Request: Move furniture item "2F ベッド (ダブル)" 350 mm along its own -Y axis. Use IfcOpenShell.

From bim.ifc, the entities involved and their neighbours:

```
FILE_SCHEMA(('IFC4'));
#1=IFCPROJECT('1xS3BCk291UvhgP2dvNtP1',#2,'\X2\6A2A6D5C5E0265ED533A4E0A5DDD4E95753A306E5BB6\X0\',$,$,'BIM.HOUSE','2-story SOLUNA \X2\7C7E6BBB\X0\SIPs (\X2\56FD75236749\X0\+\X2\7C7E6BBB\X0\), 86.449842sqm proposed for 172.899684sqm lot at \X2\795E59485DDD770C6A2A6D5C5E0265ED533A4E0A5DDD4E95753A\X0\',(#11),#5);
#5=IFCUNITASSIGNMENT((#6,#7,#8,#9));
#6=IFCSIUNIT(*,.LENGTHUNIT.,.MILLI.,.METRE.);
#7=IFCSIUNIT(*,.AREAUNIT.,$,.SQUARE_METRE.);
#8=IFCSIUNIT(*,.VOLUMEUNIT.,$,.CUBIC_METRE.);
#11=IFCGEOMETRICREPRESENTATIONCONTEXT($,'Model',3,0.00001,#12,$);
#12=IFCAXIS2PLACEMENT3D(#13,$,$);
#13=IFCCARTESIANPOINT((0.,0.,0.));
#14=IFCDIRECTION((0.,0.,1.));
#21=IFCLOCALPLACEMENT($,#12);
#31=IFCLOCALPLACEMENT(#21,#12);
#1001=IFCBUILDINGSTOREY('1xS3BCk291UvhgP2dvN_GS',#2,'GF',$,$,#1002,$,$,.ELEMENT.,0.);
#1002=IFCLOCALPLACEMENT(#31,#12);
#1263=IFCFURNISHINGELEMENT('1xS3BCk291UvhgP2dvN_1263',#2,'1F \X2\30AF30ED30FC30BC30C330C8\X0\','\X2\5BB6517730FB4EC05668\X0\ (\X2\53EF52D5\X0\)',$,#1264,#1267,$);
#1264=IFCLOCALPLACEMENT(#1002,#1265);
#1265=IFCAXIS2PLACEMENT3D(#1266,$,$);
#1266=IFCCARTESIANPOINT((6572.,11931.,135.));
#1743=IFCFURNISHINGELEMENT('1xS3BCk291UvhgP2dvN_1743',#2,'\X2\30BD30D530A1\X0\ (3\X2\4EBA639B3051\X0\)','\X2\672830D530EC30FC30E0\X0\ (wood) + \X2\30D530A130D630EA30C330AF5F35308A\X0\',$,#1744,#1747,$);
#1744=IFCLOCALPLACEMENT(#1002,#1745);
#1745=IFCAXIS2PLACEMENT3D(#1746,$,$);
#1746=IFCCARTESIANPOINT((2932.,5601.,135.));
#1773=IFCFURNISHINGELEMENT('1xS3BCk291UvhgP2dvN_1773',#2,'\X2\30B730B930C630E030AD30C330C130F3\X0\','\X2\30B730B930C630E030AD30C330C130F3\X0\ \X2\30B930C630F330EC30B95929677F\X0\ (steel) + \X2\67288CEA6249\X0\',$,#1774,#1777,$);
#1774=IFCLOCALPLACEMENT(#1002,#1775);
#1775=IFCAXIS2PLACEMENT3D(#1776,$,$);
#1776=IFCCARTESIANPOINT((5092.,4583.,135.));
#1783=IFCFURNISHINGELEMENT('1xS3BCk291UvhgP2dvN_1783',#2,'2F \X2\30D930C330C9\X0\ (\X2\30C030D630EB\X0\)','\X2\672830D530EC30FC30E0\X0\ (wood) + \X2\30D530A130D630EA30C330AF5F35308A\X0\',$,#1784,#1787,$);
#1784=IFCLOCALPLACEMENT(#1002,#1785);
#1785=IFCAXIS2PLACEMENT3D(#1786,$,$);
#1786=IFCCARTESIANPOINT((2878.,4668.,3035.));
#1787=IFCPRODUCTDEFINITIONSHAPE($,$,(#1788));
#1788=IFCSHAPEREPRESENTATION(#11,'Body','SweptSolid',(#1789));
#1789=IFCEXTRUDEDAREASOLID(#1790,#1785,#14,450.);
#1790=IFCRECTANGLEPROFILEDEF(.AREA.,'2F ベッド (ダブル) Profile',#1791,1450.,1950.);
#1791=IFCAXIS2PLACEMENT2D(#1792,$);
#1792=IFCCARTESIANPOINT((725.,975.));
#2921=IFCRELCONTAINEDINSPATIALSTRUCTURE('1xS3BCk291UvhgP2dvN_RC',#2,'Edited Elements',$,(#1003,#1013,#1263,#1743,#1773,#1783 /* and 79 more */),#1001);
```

```python
import ifcopenshell
import ifcopenshell.api.geometry
import ifcopenshell.util.placement

model = ifcopenshell.open("bim.ifc")

item = model.by_guid("1xS3BCk291UvhgP2dvN_1783")
matrix = ifcopenshell.util.placement.get_local_placement(item.ObjectPlacement)
matrix[:3, 3] -= matrix[:3, 1] * 350.0
ifcopenshell.api.geometry.edit_object_placement(model, product=item, matrix=matrix, is_si=False)

print(ifcopenshell.util.placement.get_local_placement(item.ObjectPlacement).round(3) + 0.0)

model.write("bim_edited.ifc")
```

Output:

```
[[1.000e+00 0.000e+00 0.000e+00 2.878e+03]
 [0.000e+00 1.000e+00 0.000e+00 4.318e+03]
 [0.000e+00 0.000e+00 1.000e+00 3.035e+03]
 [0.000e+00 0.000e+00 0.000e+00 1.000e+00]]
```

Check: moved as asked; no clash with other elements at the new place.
